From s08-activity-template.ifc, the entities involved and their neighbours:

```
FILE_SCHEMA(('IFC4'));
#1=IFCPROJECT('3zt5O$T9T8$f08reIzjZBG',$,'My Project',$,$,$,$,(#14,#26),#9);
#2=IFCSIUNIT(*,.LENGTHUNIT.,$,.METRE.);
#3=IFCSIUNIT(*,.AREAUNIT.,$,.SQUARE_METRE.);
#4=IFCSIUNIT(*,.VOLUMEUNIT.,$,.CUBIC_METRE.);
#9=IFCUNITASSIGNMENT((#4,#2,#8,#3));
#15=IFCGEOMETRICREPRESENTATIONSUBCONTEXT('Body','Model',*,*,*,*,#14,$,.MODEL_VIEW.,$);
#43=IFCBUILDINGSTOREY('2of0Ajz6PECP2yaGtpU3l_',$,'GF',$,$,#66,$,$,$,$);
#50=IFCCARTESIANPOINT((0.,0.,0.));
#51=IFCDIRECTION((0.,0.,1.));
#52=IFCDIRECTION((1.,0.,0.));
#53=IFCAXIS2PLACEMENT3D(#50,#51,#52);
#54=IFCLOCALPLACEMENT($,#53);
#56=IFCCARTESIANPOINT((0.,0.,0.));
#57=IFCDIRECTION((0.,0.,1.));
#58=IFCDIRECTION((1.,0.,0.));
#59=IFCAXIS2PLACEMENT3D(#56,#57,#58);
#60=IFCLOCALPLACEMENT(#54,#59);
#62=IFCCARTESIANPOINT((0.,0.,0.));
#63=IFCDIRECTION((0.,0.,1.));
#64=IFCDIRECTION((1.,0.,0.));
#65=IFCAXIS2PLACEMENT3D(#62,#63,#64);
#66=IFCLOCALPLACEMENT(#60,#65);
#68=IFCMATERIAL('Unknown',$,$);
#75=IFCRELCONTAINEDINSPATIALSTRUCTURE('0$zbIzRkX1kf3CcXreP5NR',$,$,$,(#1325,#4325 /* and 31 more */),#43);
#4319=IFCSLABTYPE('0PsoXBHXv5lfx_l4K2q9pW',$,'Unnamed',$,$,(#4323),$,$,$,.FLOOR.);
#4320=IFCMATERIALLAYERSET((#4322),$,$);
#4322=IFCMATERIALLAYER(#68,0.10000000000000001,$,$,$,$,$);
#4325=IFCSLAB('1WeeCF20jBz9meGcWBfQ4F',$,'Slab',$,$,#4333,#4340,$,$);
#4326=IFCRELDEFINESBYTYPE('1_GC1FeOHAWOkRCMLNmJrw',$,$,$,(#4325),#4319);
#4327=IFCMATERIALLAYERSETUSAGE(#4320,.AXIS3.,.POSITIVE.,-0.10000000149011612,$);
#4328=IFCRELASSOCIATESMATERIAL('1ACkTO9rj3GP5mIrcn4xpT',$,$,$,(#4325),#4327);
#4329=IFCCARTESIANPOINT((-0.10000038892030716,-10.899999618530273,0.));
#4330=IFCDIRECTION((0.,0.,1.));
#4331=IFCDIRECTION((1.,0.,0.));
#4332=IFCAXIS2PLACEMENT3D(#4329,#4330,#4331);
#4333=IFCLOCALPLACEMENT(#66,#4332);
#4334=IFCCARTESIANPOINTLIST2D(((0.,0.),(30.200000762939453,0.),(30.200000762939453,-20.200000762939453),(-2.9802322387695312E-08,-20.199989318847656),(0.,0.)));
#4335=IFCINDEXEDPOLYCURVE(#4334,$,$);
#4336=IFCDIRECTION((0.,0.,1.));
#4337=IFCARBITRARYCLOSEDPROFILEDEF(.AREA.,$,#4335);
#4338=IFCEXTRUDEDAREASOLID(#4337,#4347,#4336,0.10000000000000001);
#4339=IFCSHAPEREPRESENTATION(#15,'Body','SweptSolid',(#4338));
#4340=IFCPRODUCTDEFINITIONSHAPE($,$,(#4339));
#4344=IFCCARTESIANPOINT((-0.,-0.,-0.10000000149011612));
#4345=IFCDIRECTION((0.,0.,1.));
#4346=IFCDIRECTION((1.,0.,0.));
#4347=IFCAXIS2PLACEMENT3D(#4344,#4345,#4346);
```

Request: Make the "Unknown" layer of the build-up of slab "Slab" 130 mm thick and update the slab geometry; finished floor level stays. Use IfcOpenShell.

```python
import ifcopenshell
import ifcopenshell.util.element
import ifcopenshell.util.representation
import ifcopenshell.util.unit

model = ifcopenshell.open("s08-activity-template.ifc")
unit_scale = ifcopenshell.util.unit.calculate_unit_scale(model)

layer_set = model.by_id(4320)
layer = next(l for l in layer_set.MaterialLayers if l.Material and l.Material.Name == "Unknown")
change = 0.13 / unit_scale - layer.LayerThickness
layer.LayerThickness += change

# Geometry does not follow the layer set by itself.
slabs = [e for e in ifcopenshell.util.element.get_elements_by_material(model, layer_set) if e.is_a("IfcSlab")]
for slab in sorted(slabs, key=lambda e: e.id()):
    body = ifcopenshell.util.representation.get_representation(slab, "Model", "Body")
    solid = body.Items[0]
    old_depth = solid.Depth
    solid.Depth += change
    # Extruded upwards: lower the start of the extrusion so the top stays.
    x, y, z = solid.Position.Location.Coordinates
    solid.Position.Location = model.createIfcCartesianPoint((x, y, z - change))
    print(slab.id(), f"{old_depth:g} -> {solid.Depth:g}")

# The layers are counted up from the underside, which has moved.
for usage in {ifcopenshell.util.element.get_material(slab) for slab in slabs}:
    usage.OffsetFromReferenceLine -= change

model.write("s08-activity-template_rev.ifc")
```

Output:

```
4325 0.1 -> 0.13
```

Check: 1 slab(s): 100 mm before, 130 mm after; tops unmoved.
